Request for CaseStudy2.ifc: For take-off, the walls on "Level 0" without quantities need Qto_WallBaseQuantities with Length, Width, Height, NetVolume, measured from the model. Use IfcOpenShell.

First a look at what the model holds.

```python
import ifcopenshell
import ifcopenshell.util.element
import ifcopenshell.util.unit

model = ifcopenshell.open("CaseStudy2.ifc")
print(model.schema)
for unit_type in ("LENGTHUNIT", "AREAUNIT", "VOLUMEUNIT"):
    print(unit_type, ifcopenshell.util.unit.calculate_unit_scale(model, unit_type))
storey = next(s for s in model.by_type("IfcBuildingStorey") if s.Name == "Level 0")
walls = [e for e in ifcopenshell.util.element.get_decomposition(storey) if e.is_a("IfcWall")]
for e in sorted(walls, key=lambda e: e.id()):
    print(e.id(), e.is_a(), e.Name, list(ifcopenshell.util.element.get_psets(e, qtos_only=True)), sep=" | ")
```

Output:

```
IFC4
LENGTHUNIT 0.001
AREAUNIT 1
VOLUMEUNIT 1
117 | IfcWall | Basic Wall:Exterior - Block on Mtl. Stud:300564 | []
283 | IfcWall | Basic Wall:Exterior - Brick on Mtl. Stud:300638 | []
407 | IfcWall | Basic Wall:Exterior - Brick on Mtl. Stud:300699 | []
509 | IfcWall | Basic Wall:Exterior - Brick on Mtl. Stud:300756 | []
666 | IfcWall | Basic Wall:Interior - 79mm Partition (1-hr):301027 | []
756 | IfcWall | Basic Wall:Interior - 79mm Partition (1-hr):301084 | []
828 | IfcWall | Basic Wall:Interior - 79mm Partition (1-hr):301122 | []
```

```python
import ifcopenshell
import ifcopenshell.api.pset
import ifcopenshell.geom
import ifcopenshell.util.element
import ifcopenshell.util.shape
import ifcopenshell.util.unit

model = ifcopenshell.open("CaseStudy2.ifc")
unit_scale = ifcopenshell.util.unit.calculate_unit_scale(model)
volume_scale = ifcopenshell.util.unit.calculate_unit_scale(model, "VOLUMEUNIT")
settings = ifcopenshell.geom.settings()

storey = next(s for s in model.by_type("IfcBuildingStorey") if s.Name == "Level 0")
walls = [e for e in ifcopenshell.util.element.get_decomposition(storey) if e.is_a("IfcWall")]

for e in sorted(walls, key=lambda e: e.id()):
    if ifcopenshell.util.element.get_psets(e, qtos_only=True, should_inherit=False):
        continue
    # Geometry comes back in metres, in the element's own axes.
    shape = ifcopenshell.geom.create_shape(settings, e)
    values = {
        "Length": ifcopenshell.util.shape.get_x(shape.geometry) / unit_scale,
        "Width": ifcopenshell.util.shape.get_y(shape.geometry) / unit_scale,
        "Height": ifcopenshell.util.shape.get_z(shape.geometry) / unit_scale,
        "NetVolume": ifcopenshell.util.shape.get_volume(shape.geometry) / volume_scale,
    }
    qto = ifcopenshell.api.pset.add_qto(model, product=e, name="Qto_WallBaseQuantities")
    ifcopenshell.api.pset.edit_qto(model, qto=qto, properties=values)
    print(e.id(), {k: round(v, 3) for k, v in values.items()})

model.write("CaseStudy2-out.ifc")
```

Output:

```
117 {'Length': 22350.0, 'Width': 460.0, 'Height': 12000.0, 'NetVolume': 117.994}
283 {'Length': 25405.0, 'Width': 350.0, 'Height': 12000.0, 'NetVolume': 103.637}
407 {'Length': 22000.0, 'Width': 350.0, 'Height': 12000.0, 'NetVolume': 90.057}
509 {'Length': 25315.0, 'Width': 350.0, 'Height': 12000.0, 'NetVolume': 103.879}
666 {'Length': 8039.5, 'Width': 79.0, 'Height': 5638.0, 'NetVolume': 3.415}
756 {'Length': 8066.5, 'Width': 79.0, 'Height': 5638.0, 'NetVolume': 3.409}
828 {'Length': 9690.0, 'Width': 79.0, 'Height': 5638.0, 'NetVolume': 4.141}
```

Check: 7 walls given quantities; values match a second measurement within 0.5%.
